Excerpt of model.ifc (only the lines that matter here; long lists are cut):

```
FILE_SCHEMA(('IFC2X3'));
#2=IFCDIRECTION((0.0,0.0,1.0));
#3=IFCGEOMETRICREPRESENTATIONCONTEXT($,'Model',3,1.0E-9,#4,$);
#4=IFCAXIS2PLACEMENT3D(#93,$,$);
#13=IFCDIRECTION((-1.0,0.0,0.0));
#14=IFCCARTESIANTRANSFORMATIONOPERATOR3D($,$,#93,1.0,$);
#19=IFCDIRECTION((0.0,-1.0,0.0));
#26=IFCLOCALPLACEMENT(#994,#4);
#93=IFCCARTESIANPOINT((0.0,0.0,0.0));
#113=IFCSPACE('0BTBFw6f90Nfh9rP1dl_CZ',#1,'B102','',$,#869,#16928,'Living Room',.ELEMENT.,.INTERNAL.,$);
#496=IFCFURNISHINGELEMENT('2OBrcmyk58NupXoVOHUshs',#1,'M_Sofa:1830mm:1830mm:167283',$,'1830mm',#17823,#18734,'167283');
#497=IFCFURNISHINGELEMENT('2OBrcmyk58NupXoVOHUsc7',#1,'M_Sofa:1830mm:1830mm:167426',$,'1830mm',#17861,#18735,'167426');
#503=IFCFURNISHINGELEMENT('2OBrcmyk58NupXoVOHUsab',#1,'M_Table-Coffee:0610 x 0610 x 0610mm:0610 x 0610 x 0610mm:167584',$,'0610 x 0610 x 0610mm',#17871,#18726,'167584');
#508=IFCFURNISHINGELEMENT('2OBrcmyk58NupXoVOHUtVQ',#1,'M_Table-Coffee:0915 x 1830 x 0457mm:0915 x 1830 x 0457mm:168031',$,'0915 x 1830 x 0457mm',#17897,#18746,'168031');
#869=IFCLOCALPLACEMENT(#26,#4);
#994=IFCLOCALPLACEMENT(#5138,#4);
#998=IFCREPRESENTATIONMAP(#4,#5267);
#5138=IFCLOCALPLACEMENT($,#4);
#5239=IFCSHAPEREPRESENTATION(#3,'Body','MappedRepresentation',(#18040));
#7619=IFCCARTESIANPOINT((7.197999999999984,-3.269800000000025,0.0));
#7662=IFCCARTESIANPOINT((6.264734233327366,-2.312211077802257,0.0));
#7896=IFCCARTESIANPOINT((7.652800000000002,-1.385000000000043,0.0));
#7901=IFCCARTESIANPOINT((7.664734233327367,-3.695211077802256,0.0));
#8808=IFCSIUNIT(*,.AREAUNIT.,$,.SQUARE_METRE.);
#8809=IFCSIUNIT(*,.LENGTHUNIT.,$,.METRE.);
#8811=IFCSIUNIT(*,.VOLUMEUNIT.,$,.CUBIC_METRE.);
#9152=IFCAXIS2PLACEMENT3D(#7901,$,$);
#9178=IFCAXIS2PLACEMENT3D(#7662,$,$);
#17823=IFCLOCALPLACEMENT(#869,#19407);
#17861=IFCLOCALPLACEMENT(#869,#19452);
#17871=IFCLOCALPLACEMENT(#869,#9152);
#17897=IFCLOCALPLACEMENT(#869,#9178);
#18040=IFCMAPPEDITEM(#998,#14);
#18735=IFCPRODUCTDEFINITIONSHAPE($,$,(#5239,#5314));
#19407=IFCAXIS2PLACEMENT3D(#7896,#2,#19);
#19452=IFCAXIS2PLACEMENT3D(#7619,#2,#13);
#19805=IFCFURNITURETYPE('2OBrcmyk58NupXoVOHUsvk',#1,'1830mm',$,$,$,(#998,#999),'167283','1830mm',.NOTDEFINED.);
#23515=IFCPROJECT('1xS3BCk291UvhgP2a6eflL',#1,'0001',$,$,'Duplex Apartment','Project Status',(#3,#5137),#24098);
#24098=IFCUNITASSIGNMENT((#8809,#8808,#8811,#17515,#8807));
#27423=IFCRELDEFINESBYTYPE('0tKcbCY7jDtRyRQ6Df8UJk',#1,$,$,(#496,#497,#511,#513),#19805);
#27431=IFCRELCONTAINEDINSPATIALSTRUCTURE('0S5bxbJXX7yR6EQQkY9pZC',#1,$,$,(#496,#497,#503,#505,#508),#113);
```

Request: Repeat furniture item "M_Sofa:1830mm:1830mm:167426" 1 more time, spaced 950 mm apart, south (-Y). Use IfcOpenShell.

```python
import numpy as np
import ifcopenshell
import ifcopenshell.api.geometry
import ifcopenshell.api.root
import ifcopenshell.util.element
import ifcopenshell.util.placement
import ifcopenshell.util.unit

model = ifcopenshell.open("model.ifc")
unit_scale = ifcopenshell.util.unit.calculate_unit_scale(model)


def reuse_history(source, copy):
    """copy_class also copies each property set's owner history, people and application; keep the originals."""
    for rel in copy.IsDefinedBy:
        if rel.is_a("IfcRelDefinesByProperties") and (history := rel.RelatingPropertyDefinition.OwnerHistory):
            rel.RelatingPropertyDefinition.OwnerHistory = source.OwnerHistory
            ifcopenshell.util.element.remove_deep2(model, history)


source = model.by_guid("2OBrcmyk58NupXoVOHUsc7")
base = ifcopenshell.util.placement.get_local_placement(source.ObjectPlacement)
step = np.array([0.0, -1.0, 0.0]) * 0.95 / unit_scale

for i in range(1, 2):
    copy = ifcopenshell.api.root.copy_class(model, product=source)
    copy.Representation = ifcopenshell.util.element.copy_deep(
        model, source.Representation, exclude=["IfcGeometricRepresentationContext", "IfcRepresentationMap"]
    )
    copy.Name = "M_Sofa:1830mm:1830mm"
    copy.Tag = None
    reuse_history(source, copy)
    matrix = base.copy()
    matrix[:3, 3] += i * step
    print("added at", matrix[:3, 3].round(3) + 0.0)
    ifcopenshell.api.geometry.edit_object_placement(model, product=copy, matrix=matrix, is_si=False)

model.write("model_rev.ifc")
```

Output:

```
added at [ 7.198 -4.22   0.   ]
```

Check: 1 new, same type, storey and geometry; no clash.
